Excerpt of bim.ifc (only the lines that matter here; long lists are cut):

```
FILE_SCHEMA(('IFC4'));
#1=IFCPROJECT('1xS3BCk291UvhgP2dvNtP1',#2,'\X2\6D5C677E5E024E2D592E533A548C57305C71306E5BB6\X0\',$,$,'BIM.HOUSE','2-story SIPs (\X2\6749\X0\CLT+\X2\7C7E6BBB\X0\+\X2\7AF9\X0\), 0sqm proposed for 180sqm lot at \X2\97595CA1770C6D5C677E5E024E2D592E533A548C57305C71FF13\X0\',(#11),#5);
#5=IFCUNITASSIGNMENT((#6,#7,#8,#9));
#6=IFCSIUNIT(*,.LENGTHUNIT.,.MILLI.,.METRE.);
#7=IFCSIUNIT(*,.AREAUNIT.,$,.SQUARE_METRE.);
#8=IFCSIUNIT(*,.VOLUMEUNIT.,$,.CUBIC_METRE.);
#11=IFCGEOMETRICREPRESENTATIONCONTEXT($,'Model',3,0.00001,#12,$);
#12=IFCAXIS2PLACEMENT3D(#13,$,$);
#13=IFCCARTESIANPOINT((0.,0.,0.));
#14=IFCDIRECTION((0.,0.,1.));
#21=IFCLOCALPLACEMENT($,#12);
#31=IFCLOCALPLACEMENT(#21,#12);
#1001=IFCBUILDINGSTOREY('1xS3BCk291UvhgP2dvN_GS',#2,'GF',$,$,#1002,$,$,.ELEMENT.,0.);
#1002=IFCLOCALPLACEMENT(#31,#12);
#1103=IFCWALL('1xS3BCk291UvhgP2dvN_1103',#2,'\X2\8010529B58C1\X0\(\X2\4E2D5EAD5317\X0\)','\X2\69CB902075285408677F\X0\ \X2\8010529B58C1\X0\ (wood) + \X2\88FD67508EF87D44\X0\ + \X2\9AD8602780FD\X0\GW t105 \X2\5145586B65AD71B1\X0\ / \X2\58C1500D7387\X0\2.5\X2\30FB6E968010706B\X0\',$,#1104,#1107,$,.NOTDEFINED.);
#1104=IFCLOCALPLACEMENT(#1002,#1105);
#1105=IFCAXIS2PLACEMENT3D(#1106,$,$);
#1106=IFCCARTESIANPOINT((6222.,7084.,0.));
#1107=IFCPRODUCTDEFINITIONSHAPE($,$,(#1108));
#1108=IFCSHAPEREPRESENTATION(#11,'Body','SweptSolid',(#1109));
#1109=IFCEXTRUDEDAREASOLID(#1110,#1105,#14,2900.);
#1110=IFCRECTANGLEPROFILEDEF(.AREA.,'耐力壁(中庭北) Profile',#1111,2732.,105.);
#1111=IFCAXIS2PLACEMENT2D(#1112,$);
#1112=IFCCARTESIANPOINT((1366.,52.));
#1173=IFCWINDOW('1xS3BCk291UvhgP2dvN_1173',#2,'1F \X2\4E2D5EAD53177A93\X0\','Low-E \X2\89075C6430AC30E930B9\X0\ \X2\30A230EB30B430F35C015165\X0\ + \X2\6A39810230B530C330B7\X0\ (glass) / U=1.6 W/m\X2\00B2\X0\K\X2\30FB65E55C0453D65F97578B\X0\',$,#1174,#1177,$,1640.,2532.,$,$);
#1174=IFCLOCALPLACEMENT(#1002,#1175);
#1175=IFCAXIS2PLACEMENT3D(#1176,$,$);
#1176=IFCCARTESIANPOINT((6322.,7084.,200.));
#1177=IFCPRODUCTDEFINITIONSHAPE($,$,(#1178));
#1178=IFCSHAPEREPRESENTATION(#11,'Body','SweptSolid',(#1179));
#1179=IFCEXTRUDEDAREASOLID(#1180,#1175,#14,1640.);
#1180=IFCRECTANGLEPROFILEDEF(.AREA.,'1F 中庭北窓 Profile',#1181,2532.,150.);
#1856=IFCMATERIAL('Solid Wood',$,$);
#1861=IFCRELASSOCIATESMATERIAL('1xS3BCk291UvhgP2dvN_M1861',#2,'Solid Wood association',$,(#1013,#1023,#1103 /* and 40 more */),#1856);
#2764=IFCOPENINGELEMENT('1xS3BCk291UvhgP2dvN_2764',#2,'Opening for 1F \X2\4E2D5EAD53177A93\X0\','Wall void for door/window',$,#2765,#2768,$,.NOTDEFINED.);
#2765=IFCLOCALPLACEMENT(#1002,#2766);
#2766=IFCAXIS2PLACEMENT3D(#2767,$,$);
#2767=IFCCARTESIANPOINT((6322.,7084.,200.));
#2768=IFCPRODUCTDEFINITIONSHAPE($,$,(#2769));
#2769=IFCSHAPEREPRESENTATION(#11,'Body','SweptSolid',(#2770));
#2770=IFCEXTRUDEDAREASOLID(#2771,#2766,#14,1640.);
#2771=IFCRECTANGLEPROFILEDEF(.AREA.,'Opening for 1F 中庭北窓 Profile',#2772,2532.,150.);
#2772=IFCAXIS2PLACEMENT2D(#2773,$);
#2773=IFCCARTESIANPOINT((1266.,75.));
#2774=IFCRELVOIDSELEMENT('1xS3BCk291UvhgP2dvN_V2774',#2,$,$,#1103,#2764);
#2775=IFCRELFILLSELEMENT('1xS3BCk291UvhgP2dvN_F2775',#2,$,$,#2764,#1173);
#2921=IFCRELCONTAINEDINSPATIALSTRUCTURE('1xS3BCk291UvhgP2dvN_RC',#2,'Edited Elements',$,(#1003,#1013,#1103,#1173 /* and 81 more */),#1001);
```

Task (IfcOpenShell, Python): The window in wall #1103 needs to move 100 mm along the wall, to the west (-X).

```python
import ifcopenshell
import ifcopenshell.api.geometry
import ifcopenshell.util.placement
import ifcopenshell.util.unit

model = ifcopenshell.open("bim.ifc")
unit_scale = ifcopenshell.util.unit.calculate_unit_scale(model)

window = model.by_guid("1xS3BCk291UvhgP2dvN_1173")
opening = window.FillsVoids[0].RelatingOpeningElement
wall = opening.VoidsElements[0].RelatingBuildingElement

wall_matrix = ifcopenshell.util.placement.get_local_placement(wall.ObjectPlacement)
shift = wall_matrix[:3, 0] * -0.1 / unit_scale
before = ifcopenshell.util.placement.get_local_placement(window.ObjectPlacement)[:3, 3].copy()

# The window is not placed relative to its opening, so move both.
for product in (opening, window):
    matrix = ifcopenshell.util.placement.get_local_placement(product.ObjectPlacement)
    matrix[:3, 3] += shift
    ifcopenshell.api.geometry.edit_object_placement(model, product=product, matrix=matrix, is_si=False)

after = ifcopenshell.util.placement.get_local_placement(window.ObjectPlacement)[:3, 3]
print("window moved by", (after - before).round(3) + 0.0)

model.write("bim_edited.ifc")
```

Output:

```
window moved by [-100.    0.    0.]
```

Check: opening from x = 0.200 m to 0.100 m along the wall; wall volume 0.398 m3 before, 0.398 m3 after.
